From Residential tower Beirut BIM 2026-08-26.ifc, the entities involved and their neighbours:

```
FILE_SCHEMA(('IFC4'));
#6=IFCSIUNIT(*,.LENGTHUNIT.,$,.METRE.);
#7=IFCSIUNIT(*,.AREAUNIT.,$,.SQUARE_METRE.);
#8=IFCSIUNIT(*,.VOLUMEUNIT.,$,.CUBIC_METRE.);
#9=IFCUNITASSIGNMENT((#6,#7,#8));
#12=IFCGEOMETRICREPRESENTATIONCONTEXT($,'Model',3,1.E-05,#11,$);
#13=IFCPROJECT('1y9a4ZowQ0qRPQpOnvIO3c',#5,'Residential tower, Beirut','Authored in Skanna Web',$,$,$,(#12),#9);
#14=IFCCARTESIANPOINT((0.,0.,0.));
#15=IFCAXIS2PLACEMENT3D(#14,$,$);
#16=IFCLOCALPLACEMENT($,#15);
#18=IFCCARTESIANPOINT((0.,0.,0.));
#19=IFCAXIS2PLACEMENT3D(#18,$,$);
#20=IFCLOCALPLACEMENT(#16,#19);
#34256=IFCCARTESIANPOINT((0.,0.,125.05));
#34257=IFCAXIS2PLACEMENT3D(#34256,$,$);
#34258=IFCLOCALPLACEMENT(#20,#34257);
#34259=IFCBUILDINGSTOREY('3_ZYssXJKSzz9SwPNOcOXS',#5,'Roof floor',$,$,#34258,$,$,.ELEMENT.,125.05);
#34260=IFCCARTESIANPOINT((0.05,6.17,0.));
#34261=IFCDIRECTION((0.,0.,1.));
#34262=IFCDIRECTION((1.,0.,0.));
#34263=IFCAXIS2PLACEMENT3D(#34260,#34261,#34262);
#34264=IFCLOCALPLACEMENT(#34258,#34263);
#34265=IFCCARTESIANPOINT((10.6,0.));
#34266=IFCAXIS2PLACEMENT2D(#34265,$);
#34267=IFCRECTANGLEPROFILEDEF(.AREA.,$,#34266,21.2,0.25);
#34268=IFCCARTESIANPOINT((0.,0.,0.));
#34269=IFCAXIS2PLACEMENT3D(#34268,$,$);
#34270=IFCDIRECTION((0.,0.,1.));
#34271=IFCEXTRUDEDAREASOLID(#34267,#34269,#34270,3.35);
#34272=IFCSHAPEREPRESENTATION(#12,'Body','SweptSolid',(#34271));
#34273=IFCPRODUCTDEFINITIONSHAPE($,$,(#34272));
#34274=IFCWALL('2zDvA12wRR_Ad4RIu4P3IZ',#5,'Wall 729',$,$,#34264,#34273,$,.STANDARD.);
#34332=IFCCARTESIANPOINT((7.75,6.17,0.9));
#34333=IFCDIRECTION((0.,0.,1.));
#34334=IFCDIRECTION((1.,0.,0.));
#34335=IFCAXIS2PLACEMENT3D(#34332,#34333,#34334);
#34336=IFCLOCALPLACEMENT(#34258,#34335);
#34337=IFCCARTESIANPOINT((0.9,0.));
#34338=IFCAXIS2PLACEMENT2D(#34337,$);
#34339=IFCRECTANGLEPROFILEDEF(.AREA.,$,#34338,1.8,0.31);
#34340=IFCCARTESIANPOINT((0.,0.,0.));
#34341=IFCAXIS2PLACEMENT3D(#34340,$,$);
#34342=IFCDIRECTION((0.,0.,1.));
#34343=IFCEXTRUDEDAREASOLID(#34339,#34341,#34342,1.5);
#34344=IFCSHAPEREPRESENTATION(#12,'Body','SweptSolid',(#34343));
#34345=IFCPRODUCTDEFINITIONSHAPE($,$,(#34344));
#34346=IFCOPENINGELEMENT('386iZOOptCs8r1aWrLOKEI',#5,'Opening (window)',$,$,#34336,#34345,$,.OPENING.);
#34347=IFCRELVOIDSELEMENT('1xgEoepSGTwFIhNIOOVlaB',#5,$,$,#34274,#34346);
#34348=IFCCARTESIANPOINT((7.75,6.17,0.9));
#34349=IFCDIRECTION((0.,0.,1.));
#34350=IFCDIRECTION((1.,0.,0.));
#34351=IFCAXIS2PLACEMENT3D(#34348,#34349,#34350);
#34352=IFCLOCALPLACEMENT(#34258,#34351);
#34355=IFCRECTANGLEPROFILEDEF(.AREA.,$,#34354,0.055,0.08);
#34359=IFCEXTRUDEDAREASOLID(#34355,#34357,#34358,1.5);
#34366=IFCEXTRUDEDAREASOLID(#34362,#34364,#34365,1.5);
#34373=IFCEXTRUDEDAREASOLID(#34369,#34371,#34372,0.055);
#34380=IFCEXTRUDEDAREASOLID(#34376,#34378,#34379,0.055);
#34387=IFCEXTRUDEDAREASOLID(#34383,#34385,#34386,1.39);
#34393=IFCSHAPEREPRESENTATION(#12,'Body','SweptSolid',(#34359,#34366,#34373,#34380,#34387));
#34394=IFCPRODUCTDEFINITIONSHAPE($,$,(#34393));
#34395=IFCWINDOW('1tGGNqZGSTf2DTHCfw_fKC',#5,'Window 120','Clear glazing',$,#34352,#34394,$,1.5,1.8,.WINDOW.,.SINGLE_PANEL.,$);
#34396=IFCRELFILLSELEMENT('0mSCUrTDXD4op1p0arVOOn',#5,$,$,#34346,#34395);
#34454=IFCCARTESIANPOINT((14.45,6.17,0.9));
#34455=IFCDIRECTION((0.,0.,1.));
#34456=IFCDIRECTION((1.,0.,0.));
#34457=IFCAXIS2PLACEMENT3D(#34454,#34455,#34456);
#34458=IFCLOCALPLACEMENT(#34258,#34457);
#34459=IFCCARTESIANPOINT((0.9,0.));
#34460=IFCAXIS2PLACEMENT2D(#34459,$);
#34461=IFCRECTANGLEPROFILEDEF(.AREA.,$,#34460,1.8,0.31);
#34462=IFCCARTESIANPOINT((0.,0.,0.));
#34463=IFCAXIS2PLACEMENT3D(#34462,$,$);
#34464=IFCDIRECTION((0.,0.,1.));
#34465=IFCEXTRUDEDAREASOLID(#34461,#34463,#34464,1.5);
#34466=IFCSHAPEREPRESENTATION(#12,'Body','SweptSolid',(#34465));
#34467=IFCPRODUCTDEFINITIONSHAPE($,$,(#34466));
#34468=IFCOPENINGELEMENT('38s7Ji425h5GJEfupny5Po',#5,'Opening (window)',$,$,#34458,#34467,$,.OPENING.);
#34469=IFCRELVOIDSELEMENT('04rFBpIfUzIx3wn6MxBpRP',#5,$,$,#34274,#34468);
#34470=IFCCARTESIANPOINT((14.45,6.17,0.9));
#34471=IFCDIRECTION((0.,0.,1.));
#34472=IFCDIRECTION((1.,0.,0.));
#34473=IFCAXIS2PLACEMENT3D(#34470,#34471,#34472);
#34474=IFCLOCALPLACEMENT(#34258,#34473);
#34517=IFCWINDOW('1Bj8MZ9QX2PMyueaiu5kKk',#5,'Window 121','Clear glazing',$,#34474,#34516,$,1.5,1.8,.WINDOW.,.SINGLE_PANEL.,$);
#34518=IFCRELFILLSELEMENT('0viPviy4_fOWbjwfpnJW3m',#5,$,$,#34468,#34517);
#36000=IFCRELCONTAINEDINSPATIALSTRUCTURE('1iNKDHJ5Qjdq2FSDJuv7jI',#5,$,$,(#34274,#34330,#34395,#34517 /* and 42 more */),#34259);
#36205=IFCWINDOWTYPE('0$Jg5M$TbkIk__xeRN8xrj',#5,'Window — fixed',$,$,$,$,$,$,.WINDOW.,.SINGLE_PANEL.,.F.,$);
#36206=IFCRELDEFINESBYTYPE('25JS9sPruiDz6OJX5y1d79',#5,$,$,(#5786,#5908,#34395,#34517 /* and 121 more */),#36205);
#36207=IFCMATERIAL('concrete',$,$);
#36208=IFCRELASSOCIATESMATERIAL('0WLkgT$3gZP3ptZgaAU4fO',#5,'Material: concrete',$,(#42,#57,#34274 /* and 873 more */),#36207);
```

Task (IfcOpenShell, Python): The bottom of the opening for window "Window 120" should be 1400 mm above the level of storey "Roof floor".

```python
import numpy as np
import ifcopenshell
import ifcopenshell.api.geometry
import ifcopenshell.geom
import ifcopenshell.util.element
import ifcopenshell.util.placement
import ifcopenshell.util.shape
import ifcopenshell.util.unit

model = ifcopenshell.open("Residential tower Beirut BIM 2026-08-26.ifc")
unit_scale = ifcopenshell.util.unit.calculate_unit_scale(model)

window = model.by_guid("1tGGNqZGSTf2DTHCfw_fKC")
opening = window.FillsVoids[0].RelatingOpeningElement
storey = ifcopenshell.util.element.get_container(window, ifc_class="IfcBuildingStorey")
level = ifcopenshell.util.placement.get_local_placement(storey.ObjectPlacement)[2, 3]

# The opening's origin need not be at the sill, so measure its lowest point.
shape = ifcopenshell.geom.create_shape(ifcopenshell.geom.settings(), opening)
bottom = ifcopenshell.util.shape.get_shape_bottom_elevation(shape, shape.geometry) / unit_scale
dz = level + 1.4 - bottom

shift = np.array([0.0, 0.0, dz])
# The window is not placed relative to its opening, so move both.
for product in (opening, window):
    matrix = ifcopenshell.util.placement.get_local_placement(product.ObjectPlacement)
    matrix[:3, 3] += shift
    ifcopenshell.api.geometry.edit_object_placement(model, product=product, matrix=matrix, is_si=False)

print(f"moved by {dz * unit_scale:+.3f} m")

model.write("Residential tower Beirut BIM 2026-08-26_rev.ifc")
```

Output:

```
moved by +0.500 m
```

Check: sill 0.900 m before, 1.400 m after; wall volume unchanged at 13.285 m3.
